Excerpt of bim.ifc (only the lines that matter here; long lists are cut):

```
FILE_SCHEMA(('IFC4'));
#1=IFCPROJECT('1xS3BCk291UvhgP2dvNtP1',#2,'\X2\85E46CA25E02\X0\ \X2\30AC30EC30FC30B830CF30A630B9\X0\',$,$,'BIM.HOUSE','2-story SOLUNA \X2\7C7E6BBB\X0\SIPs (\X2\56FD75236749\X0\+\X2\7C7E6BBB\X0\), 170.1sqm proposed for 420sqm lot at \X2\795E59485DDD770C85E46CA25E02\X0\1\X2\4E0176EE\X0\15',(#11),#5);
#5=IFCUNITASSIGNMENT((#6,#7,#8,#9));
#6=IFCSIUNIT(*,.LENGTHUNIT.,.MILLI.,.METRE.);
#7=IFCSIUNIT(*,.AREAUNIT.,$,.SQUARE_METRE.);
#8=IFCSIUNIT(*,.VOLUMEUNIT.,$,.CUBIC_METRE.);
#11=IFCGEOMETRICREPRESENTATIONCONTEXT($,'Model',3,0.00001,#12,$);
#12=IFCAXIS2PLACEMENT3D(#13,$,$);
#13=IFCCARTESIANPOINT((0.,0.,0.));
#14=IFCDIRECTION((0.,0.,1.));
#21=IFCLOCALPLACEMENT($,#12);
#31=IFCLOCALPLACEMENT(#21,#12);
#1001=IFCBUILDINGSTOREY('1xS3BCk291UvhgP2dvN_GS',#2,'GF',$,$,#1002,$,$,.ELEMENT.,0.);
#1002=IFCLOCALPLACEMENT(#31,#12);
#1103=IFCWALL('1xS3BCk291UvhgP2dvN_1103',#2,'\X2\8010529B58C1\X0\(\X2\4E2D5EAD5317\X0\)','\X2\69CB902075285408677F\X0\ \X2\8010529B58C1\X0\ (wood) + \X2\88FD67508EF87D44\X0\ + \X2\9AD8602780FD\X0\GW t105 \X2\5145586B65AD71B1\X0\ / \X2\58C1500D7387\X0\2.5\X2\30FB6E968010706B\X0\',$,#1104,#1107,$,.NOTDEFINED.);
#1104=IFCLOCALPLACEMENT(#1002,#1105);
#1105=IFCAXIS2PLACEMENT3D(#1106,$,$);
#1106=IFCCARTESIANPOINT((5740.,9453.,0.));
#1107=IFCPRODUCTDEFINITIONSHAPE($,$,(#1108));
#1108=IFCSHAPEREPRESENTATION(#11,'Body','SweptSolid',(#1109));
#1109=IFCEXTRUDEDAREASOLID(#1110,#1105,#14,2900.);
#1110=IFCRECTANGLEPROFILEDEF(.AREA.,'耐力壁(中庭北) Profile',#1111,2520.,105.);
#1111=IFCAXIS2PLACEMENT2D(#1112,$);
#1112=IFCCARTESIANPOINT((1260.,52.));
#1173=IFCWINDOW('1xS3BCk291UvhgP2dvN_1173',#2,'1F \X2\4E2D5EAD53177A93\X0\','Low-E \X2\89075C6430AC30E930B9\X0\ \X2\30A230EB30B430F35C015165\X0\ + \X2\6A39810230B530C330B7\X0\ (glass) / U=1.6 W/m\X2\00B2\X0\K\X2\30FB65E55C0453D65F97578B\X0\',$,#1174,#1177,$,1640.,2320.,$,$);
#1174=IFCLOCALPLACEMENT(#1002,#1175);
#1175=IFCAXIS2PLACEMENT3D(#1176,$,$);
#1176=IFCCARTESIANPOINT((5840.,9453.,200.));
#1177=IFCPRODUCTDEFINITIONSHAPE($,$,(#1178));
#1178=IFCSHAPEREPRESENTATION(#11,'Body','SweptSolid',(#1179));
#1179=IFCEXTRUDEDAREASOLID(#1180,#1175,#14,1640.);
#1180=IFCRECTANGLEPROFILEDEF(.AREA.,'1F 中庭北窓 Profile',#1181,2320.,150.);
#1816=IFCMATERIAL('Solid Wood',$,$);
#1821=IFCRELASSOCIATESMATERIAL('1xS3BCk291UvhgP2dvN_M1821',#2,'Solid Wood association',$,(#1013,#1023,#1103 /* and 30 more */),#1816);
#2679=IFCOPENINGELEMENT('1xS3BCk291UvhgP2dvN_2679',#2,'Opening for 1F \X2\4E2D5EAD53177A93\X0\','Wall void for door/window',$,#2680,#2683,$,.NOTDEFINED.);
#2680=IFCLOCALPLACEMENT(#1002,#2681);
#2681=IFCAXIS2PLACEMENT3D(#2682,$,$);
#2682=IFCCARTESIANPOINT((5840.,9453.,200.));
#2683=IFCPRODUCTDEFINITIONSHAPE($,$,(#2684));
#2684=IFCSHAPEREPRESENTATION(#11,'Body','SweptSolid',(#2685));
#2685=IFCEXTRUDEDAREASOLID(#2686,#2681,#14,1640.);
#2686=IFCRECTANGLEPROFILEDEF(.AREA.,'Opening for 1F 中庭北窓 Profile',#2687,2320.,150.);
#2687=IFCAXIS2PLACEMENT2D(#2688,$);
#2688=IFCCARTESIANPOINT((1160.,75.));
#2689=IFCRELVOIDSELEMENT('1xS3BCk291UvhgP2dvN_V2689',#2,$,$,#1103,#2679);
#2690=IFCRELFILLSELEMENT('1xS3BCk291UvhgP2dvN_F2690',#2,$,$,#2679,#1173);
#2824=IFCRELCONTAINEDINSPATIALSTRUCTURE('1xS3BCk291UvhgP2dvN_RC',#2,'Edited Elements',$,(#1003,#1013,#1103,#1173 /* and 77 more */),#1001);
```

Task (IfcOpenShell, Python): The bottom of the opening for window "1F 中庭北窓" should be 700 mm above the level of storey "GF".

```python
import numpy as np
import ifcopenshell
import ifcopenshell.api.geometry
import ifcopenshell.geom
import ifcopenshell.util.element
import ifcopenshell.util.placement
import ifcopenshell.util.shape
import ifcopenshell.util.unit

model = ifcopenshell.open("bim.ifc")
unit_scale = ifcopenshell.util.unit.calculate_unit_scale(model)

window = model.by_guid("1xS3BCk291UvhgP2dvN_1173")
opening = window.FillsVoids[0].RelatingOpeningElement
storey = ifcopenshell.util.element.get_container(window, ifc_class="IfcBuildingStorey")
level = ifcopenshell.util.placement.get_local_placement(storey.ObjectPlacement)[2, 3]

# The opening's origin need not be at the sill, so measure its lowest point.
shape = ifcopenshell.geom.create_shape(ifcopenshell.geom.settings(), opening)
bottom = ifcopenshell.util.shape.get_shape_bottom_elevation(shape, shape.geometry) / unit_scale
dz = level + 0.7 / unit_scale - bottom

shift = np.array([0.0, 0.0, dz])
# The window is not placed relative to its opening, so move both.
for product in (opening, window):
    matrix = ifcopenshell.util.placement.get_local_placement(product.ObjectPlacement)
    matrix[:3, 3] += shift
    ifcopenshell.api.geometry.edit_object_placement(model, product=product, matrix=matrix, is_si=False)

print(f"moved by {dz * unit_scale:+.3f} m")

model.write("bim_rev.ifc")
```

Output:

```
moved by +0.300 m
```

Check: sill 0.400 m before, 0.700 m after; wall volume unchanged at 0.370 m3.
